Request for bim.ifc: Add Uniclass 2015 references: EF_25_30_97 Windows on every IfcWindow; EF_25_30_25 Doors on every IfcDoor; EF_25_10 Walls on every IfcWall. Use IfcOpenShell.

First a look at what the model holds.

```python
import ifcopenshell

model = ifcopenshell.open("bim.ifc")
print(model.schema)
print("classifications:", [c.Name for c in model.by_type("IfcClassification")])
for ifc_class in ("IfcDoor", "IfcRoof", "IfcStair", "IfcWall", "IfcWindow"):
    print(ifc_class, len(model.by_type(ifc_class)))
```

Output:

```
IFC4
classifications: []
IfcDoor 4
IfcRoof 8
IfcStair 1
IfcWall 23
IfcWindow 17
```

```python
import ifcopenshell
import ifcopenshell.api.classification

model = ifcopenshell.open("bim.ifc")

system = ifcopenshell.api.classification.add_classification(model, classification="Uniclass 2015")

codes = {
    "IfcWindow": ("EF_25_30_97", "Windows"),
    "IfcDoor": ("EF_25_30_25", "Doors"),
    "IfcWall": ("EF_25_10", "Walls"),
}
for ifc_class, (code, name) in codes.items():
    products = model.by_type(ifc_class)
    ifcopenshell.api.classification.add_reference(
        model, products=products, classification=system, identification=code, name=name
    )
    print(code, len(products))

model.write("bim_updated.ifc")
```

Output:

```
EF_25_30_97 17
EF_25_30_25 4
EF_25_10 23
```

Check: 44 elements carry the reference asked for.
